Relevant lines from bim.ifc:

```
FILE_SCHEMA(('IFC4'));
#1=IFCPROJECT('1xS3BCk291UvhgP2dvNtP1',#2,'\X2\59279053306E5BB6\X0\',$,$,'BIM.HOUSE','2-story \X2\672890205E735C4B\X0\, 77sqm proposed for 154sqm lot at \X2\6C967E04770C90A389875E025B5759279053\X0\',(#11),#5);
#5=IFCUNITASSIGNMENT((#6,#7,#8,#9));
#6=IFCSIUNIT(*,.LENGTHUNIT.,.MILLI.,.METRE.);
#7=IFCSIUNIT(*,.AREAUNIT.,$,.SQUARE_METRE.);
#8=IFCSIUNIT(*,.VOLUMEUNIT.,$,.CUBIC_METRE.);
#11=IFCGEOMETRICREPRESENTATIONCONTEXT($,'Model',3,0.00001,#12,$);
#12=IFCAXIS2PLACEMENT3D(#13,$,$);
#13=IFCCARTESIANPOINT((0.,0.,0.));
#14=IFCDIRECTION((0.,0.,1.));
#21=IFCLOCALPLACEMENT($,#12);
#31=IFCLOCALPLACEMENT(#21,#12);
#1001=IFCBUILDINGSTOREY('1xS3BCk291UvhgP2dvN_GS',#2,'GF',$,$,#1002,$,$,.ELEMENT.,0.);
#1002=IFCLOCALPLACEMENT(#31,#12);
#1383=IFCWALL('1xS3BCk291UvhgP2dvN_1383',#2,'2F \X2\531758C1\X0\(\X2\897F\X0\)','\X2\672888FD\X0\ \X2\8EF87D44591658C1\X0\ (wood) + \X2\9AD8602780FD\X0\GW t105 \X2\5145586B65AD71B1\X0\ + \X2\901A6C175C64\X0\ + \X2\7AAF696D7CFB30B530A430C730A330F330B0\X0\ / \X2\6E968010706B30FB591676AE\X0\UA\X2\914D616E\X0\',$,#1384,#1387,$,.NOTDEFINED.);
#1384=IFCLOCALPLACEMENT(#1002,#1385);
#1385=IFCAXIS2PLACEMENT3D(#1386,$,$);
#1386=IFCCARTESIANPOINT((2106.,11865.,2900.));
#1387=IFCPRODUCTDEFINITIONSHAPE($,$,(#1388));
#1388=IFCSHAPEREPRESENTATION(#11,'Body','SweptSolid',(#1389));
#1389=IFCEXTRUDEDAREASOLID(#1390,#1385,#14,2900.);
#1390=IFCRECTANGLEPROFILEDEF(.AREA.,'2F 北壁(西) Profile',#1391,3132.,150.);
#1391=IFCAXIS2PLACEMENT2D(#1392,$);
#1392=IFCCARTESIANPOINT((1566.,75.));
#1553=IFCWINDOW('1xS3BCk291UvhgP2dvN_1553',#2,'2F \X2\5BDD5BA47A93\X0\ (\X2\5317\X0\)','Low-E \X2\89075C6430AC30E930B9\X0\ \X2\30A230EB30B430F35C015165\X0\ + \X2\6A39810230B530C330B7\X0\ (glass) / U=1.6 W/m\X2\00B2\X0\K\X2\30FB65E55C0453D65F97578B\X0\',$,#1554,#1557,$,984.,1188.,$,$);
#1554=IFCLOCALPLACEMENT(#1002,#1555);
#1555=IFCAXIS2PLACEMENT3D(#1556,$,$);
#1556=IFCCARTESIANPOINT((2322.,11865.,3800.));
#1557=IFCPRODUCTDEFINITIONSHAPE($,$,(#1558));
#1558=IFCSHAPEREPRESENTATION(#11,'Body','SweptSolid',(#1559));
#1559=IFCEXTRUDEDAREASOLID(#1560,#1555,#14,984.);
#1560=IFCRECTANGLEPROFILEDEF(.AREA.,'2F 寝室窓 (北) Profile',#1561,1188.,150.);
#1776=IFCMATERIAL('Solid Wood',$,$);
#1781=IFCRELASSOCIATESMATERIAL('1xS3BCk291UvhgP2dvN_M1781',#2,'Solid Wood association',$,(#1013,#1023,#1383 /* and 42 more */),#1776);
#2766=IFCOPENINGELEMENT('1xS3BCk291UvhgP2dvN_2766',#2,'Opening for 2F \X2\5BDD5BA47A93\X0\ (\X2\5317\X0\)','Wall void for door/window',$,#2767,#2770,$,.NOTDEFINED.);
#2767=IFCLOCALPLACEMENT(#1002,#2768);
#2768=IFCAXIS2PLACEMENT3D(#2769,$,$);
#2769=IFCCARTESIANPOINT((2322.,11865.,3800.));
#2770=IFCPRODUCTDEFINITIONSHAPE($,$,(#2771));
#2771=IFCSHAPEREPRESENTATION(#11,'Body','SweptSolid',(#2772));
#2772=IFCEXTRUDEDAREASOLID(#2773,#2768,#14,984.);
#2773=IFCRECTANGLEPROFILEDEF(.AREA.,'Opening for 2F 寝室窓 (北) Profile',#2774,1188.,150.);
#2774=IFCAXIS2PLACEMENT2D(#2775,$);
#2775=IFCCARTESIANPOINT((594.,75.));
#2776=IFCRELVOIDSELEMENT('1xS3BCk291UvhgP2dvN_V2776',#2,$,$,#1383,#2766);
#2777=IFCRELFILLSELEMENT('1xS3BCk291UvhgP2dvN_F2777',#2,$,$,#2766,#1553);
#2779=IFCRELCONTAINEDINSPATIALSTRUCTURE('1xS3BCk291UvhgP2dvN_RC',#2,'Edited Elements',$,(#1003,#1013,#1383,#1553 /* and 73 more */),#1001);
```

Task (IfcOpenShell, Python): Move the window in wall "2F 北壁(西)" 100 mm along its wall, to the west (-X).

```python
import ifcopenshell
import ifcopenshell.api.geometry
import ifcopenshell.util.placement

model = ifcopenshell.open("bim.ifc")

window = model.by_guid("1xS3BCk291UvhgP2dvN_1553")
opening = window.FillsVoids[0].RelatingOpeningElement
wall = opening.VoidsElements[0].RelatingBuildingElement

wall_matrix = ifcopenshell.util.placement.get_local_placement(wall.ObjectPlacement)
shift = wall_matrix[:3, 0] * -100.0
before = ifcopenshell.util.placement.get_local_placement(window.ObjectPlacement)[:3, 3].copy()

# The window is not placed relative to its opening, so move both.
for product in (opening, window):
    matrix = ifcopenshell.util.placement.get_local_placement(product.ObjectPlacement)
    matrix[:3, 3] += shift
    ifcopenshell.api.geometry.edit_object_placement(model, product=product, matrix=matrix, is_si=False)

after = ifcopenshell.util.placement.get_local_placement(window.ObjectPlacement)[:3, 3]
print("window moved by", (after - before).round(3) + 0.0)

model.write("bim-out.ifc")
```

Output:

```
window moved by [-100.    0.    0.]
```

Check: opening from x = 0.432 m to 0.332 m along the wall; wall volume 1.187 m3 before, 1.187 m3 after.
